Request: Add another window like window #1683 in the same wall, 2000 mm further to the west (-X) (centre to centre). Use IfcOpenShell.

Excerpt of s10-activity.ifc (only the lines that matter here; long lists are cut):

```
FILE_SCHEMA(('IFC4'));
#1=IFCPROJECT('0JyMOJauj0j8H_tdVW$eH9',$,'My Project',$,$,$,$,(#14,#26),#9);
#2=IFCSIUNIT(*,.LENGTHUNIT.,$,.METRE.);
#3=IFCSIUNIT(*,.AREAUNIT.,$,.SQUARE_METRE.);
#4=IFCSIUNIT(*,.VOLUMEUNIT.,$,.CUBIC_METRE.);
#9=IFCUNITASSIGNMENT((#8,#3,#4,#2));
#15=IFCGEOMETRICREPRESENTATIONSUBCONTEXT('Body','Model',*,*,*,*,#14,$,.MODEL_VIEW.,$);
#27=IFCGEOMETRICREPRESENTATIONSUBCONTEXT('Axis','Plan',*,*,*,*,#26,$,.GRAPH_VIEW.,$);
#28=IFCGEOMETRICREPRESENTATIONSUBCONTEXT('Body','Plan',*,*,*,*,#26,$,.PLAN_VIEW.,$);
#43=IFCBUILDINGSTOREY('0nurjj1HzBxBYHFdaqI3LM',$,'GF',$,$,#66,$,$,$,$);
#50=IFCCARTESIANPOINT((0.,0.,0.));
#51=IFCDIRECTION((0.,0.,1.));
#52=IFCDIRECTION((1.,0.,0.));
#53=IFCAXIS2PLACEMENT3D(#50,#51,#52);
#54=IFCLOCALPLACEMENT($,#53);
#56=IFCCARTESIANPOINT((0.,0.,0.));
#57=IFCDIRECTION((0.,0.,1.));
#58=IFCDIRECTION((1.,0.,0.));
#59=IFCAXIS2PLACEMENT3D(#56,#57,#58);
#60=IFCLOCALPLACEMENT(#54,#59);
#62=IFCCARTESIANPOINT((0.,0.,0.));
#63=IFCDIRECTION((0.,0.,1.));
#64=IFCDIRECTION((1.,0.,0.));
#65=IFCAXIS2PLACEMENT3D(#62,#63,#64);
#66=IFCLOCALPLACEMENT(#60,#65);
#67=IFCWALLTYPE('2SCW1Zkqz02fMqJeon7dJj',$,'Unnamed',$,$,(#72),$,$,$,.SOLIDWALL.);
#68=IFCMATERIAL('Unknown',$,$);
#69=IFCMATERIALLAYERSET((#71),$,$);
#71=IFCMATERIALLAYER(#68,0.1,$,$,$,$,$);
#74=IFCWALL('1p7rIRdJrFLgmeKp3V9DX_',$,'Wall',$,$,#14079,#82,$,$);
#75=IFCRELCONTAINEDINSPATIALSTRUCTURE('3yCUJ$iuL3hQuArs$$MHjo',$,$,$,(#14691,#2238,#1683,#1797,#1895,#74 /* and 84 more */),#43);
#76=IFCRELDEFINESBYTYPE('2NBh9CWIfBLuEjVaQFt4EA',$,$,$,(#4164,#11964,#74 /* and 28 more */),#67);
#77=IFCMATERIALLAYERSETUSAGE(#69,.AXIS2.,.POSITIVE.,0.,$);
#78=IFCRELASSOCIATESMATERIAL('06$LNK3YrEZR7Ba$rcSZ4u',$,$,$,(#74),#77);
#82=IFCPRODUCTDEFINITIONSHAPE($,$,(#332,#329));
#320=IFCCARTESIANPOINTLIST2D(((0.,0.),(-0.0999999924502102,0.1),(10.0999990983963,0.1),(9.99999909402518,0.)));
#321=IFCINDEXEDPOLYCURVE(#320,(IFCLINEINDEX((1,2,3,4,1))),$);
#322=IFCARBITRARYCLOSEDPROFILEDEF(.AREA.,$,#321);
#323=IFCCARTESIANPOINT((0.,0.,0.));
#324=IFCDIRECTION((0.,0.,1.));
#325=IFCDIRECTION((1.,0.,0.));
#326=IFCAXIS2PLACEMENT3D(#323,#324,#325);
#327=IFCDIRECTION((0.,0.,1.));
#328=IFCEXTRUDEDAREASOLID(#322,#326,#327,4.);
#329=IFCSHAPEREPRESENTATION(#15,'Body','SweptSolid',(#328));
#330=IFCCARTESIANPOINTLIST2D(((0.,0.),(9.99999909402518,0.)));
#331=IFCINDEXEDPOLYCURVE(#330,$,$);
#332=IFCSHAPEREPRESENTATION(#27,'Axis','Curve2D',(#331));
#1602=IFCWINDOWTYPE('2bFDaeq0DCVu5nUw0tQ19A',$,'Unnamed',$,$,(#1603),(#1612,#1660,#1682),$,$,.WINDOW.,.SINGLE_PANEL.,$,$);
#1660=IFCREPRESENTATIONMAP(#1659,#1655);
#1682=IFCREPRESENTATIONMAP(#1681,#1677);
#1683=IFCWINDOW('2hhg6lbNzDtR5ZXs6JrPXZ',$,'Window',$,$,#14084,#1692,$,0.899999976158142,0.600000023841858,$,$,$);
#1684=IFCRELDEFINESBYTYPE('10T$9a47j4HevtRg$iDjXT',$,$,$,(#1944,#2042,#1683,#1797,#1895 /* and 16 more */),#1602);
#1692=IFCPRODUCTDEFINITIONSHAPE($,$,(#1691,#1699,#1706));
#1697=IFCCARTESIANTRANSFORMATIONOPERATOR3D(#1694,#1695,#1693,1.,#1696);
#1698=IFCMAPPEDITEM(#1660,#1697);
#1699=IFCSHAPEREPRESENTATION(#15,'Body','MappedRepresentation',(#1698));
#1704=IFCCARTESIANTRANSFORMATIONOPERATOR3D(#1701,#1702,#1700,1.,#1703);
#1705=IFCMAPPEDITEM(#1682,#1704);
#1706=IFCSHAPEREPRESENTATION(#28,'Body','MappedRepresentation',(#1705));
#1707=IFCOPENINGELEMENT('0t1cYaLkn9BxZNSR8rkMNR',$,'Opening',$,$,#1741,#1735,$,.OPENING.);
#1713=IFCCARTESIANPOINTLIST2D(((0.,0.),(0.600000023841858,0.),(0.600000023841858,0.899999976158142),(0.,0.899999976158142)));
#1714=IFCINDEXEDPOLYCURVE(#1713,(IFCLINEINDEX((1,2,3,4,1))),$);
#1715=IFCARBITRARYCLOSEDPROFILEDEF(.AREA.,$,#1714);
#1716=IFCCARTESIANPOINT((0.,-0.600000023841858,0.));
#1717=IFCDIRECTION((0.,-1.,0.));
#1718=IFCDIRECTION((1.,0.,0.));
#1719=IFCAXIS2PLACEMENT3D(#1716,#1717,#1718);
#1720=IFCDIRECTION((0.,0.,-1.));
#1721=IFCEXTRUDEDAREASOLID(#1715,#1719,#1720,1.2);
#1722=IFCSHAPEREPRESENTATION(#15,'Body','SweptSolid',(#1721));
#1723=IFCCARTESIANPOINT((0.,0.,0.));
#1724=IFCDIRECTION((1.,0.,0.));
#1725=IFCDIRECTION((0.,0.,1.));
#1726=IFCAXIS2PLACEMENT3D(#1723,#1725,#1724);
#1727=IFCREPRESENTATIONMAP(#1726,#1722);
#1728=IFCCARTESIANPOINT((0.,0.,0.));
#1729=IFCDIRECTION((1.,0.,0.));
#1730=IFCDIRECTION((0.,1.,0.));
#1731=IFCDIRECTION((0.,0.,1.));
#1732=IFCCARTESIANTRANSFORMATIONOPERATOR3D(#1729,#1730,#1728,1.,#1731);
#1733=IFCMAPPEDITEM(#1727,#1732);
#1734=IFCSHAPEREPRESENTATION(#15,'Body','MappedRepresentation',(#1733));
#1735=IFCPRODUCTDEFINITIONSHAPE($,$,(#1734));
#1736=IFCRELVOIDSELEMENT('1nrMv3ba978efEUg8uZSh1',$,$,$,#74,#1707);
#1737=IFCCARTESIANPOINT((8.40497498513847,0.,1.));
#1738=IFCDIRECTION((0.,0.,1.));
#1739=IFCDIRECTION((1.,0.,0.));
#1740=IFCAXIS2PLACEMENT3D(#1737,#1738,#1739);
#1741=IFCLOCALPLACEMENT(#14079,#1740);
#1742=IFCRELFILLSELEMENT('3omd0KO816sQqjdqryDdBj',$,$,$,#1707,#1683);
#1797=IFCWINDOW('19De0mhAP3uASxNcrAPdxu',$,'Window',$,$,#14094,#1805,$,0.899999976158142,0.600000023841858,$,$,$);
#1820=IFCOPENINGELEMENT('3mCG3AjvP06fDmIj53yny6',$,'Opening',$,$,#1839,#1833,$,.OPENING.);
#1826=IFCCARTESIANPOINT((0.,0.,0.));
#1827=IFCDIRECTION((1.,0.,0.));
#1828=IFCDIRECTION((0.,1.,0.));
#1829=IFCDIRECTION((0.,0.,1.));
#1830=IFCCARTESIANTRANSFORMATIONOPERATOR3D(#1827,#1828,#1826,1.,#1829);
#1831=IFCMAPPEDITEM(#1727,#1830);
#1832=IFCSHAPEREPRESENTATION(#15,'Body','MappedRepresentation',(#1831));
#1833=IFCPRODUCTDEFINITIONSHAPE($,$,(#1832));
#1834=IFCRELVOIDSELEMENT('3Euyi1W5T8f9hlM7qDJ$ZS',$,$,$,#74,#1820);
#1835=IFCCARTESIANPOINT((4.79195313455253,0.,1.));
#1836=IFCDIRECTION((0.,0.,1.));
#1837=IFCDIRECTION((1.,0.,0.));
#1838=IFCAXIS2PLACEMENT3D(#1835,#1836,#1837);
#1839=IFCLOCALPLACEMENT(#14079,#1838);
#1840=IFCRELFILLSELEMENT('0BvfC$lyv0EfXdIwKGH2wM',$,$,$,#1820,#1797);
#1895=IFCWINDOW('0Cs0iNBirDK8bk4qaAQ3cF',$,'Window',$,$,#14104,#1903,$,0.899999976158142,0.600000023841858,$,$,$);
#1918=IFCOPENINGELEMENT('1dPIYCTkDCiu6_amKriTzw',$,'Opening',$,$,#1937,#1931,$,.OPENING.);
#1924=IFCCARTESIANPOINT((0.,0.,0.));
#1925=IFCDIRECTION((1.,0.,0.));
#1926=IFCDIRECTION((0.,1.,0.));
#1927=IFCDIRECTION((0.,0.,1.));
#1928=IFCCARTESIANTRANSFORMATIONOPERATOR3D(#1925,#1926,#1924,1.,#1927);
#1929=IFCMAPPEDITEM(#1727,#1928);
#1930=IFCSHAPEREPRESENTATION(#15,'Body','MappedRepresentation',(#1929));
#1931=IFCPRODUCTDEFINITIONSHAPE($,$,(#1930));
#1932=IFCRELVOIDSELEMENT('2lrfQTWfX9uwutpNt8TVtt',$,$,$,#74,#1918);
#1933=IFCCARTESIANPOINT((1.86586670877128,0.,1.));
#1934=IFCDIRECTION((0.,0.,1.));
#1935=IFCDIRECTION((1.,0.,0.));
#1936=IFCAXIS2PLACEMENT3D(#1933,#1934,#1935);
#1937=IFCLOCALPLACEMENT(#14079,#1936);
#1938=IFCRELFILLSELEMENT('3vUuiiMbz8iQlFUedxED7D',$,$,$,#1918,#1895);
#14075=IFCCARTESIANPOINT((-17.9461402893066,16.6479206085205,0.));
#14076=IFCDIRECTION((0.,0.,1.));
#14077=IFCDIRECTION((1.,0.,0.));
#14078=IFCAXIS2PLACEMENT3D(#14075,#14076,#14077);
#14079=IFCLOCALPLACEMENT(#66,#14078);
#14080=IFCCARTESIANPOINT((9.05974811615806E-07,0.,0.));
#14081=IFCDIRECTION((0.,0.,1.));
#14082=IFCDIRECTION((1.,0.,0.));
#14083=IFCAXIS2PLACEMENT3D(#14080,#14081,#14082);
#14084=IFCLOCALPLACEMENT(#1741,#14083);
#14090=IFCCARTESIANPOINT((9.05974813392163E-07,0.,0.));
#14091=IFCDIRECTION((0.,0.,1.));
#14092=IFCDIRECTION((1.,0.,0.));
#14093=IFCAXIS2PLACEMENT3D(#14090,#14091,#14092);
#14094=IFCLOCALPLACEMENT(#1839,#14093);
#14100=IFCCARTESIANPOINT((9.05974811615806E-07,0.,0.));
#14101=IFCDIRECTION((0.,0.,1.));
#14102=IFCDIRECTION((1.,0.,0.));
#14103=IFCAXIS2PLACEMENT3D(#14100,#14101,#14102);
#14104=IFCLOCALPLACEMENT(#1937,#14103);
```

```python
import ifcopenshell
import ifcopenshell.api.feature
import ifcopenshell.api.geometry
import ifcopenshell.api.root
import ifcopenshell.geom
import ifcopenshell.util.element
import ifcopenshell.util.placement
import ifcopenshell.util.shape

model = ifcopenshell.open("s10-activity.ifc")
settings = ifcopenshell.geom.settings()


def volume(element):
    """Net volume in cubic metres, openings subtracted."""
    shape = ifcopenshell.geom.create_shape(settings, element)
    return ifcopenshell.util.shape.get_volume(shape.geometry)


window = model.by_id(1683)
opening = window.FillsVoids[0].RelatingOpeningElement
wall = opening.VoidsElements[0].RelatingBuildingElement
before = volume(wall)
shift = ifcopenshell.util.placement.get_local_placement(wall.ObjectPlacement)[:3, 0] * -2.0

# copy_class copies the void relationship, type, container and properties, but no geometry.
new_opening = ifcopenshell.api.root.copy_class(model, product=opening)
new_opening.Representation = ifcopenshell.util.element.copy_deep(
    model, opening.Representation, exclude=["IfcGeometricRepresentationContext", "IfcRepresentationMap"]
)
new_window = ifcopenshell.api.root.copy_class(model, product=window)
new_window.Representation = ifcopenshell.util.element.copy_deep(
    model, window.Representation, exclude=["IfcGeometricRepresentationContext", "IfcRepresentationMap"]
)
ifcopenshell.api.feature.add_filling(model, opening=new_opening, element=new_window)

for old, new in ((opening, new_opening), (window, new_window)):
    matrix = ifcopenshell.util.placement.get_local_placement(old.ObjectPlacement)
    matrix[:3, 3] += shift
    ifcopenshell.api.geometry.edit_object_placement(model, product=new, matrix=matrix, is_si=False)

after = volume(wall)

print(f"wall volume {before:.3f} -> {after:.3f} m3")

model.write("s10-activity_v2.ifc")
```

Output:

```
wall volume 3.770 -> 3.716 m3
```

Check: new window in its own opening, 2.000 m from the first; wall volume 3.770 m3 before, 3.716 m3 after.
